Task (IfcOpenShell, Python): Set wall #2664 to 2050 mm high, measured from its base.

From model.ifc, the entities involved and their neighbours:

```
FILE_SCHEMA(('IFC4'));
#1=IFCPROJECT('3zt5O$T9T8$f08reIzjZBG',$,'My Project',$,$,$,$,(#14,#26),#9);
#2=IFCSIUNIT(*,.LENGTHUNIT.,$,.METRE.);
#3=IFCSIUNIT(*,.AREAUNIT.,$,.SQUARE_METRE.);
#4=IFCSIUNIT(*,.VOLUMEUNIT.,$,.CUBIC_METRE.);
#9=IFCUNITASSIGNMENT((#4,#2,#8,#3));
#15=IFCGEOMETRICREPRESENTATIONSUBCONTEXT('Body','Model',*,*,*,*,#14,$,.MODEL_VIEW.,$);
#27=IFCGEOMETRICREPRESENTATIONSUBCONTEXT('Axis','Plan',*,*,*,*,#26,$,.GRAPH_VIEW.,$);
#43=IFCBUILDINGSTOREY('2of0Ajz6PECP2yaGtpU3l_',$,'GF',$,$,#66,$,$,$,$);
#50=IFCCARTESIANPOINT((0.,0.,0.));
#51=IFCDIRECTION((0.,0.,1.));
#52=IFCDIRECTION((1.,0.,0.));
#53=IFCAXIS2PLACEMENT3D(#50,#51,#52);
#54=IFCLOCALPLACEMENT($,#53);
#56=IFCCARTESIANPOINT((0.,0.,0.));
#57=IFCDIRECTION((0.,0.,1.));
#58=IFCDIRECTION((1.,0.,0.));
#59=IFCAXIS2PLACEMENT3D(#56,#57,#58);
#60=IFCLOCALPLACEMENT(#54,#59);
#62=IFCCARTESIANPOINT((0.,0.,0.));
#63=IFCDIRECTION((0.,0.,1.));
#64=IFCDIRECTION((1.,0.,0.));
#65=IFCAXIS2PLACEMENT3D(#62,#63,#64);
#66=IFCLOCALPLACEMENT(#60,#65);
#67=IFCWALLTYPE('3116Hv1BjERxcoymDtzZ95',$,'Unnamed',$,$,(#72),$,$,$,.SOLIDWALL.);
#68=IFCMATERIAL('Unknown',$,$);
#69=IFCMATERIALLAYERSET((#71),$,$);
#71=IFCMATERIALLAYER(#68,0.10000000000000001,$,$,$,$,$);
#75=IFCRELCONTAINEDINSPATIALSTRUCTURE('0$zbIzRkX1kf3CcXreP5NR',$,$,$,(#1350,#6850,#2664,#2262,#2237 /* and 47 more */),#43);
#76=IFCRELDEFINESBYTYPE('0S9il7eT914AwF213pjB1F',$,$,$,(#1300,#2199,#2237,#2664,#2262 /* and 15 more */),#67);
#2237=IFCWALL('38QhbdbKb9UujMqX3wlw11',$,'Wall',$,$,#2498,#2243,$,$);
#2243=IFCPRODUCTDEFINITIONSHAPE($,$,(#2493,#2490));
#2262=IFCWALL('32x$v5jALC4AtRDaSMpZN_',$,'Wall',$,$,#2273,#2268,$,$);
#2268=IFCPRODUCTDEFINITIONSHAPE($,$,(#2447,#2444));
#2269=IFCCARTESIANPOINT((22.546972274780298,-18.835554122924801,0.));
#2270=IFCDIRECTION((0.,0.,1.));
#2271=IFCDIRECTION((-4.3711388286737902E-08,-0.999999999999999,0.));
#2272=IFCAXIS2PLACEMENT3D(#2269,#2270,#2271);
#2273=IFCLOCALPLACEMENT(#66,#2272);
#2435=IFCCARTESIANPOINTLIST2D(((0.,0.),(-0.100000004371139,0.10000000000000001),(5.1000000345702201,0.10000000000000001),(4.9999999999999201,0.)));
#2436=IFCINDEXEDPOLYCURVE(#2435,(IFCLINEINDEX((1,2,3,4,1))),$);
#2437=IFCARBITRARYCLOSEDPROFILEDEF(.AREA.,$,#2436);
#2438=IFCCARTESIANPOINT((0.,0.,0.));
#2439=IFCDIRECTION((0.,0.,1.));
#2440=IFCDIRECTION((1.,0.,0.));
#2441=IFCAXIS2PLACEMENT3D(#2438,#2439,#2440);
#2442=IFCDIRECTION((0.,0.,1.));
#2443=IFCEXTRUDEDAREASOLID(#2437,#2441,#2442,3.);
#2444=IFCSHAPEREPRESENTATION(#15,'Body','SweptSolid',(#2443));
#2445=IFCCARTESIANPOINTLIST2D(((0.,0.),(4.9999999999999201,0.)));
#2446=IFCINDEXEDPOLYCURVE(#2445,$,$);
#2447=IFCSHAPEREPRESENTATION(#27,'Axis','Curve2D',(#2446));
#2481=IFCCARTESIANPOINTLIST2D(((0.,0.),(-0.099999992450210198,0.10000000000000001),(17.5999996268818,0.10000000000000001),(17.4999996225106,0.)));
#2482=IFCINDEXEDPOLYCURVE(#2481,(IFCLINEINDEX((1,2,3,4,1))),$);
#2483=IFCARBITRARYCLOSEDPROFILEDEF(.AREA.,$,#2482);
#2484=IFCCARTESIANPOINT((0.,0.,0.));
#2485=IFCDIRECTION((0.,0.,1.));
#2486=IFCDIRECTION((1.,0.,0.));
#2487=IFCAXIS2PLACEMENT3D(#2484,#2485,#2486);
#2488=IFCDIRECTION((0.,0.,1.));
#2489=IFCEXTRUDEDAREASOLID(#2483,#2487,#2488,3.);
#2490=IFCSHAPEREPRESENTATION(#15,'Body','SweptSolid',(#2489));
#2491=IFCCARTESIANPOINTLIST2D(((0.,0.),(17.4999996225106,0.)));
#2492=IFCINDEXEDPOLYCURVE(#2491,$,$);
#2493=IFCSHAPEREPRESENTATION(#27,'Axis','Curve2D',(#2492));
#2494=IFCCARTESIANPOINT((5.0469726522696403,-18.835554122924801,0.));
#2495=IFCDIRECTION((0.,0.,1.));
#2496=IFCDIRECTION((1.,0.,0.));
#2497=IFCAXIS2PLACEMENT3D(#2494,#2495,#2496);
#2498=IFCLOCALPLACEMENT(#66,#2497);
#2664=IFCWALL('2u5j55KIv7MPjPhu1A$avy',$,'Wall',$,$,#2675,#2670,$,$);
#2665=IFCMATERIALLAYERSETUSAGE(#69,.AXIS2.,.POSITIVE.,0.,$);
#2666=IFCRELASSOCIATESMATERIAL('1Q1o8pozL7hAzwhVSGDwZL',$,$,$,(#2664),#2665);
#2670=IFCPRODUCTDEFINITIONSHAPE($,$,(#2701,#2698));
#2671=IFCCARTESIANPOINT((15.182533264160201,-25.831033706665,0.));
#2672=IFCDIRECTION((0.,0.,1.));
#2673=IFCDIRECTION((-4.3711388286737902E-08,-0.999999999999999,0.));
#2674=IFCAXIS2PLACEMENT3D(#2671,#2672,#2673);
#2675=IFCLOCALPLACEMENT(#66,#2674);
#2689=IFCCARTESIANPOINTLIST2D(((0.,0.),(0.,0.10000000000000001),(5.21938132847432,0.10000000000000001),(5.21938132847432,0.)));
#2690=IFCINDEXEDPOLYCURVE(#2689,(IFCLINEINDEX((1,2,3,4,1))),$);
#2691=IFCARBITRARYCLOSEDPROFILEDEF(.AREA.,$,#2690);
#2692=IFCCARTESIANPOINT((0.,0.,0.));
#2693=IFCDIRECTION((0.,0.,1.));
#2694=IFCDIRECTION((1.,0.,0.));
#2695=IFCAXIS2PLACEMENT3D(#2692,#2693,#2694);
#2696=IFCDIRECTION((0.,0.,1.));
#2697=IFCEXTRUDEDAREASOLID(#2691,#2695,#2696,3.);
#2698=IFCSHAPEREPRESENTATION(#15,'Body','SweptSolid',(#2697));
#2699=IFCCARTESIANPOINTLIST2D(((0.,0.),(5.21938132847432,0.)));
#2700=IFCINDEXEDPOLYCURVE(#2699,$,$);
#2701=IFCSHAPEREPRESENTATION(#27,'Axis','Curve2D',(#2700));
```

```python
import ifcopenshell
import ifcopenshell.geom
import ifcopenshell.util.representation
import ifcopenshell.util.shape
import ifcopenshell.util.unit

model = ifcopenshell.open("model.ifc")
unit_scale = ifcopenshell.util.unit.calculate_unit_scale(model)
settings = ifcopenshell.geom.settings()


def volume(element):
    """Net volume in cubic metres, openings subtracted."""
    shape = ifcopenshell.geom.create_shape(settings, element)
    return ifcopenshell.util.shape.get_volume(shape.geometry)


wall = model.by_guid("2u5j55KIv7MPjPhu1A$avy")
before = volume(wall)

body = ifcopenshell.util.representation.get_representation(wall, "Model", "Body")
solid = body.Items[0]
old_height = solid.Depth
solid.Depth = 2.05 / unit_scale
after = volume(wall)

print(f"height {old_height:g} -> {solid.Depth:g}, volume {before:.3f} -> {after:.3f} m3")

model.write("model_rev.ifc")
```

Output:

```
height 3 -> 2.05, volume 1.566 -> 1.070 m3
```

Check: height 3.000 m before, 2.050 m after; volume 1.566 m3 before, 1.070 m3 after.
